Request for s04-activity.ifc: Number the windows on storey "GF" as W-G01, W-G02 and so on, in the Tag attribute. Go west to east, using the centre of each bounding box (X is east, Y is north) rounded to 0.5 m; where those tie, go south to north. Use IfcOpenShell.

First a look at what the model holds.

```python
import ifcopenshell
import ifcopenshell.util.element
import ifcopenshell.util.placement

model = ifcopenshell.open("s04-activity.ifc")
print(model.schema)
storey = next(s for s in model.by_type("IfcBuildingStorey") if s.Name == "GF")
windows = [e for e in ifcopenshell.util.element.get_decomposition(storey) if e.is_a("IfcWindow")]
for e in sorted(windows, key=lambda e: e.id()):
    origin = ifcopenshell.util.placement.get_local_placement(e.ObjectPlacement)[:3, 3]
    print(e.id(), e.Tag, e.Name, origin.round(2) + 0.0, sep=" | ")
```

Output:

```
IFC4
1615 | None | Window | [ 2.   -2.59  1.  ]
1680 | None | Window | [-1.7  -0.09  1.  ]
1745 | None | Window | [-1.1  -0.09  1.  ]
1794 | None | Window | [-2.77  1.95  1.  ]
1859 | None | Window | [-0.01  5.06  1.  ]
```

```python
import ifcopenshell
import ifcopenshell.geom
import ifcopenshell.util.element
import ifcopenshell.util.shape

model = ifcopenshell.open("s04-activity.ifc")
settings = ifcopenshell.geom.settings()
settings.set("use-world-coords", True)


def centre(element):
    shape = ifcopenshell.geom.create_shape(settings, element)
    return ifcopenshell.util.shape.get_bbox_centroid(shape.geometry)


storey = next(s for s in model.by_type("IfcBuildingStorey") if s.Name == "GF")
windows = [e for e in ifcopenshell.util.element.get_decomposition(storey) if e.is_a("IfcWindow")]

# Insertion points can sit at a corner or the storey origin, so sort by the geometry (in metres).
centres = {e: centre(e) for e in windows}
windows.sort(key=lambda e: (round(centres[e][0] / 0.5), centres[e][1]))

for i, e in enumerate(windows, start=1):
    number = f"W-G{i:02d}"
    e.Tag = number
    print(e.id(), number)

model.write("s04-activity_rev.ifc")
```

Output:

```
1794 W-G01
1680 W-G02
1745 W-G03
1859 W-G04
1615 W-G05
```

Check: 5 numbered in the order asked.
